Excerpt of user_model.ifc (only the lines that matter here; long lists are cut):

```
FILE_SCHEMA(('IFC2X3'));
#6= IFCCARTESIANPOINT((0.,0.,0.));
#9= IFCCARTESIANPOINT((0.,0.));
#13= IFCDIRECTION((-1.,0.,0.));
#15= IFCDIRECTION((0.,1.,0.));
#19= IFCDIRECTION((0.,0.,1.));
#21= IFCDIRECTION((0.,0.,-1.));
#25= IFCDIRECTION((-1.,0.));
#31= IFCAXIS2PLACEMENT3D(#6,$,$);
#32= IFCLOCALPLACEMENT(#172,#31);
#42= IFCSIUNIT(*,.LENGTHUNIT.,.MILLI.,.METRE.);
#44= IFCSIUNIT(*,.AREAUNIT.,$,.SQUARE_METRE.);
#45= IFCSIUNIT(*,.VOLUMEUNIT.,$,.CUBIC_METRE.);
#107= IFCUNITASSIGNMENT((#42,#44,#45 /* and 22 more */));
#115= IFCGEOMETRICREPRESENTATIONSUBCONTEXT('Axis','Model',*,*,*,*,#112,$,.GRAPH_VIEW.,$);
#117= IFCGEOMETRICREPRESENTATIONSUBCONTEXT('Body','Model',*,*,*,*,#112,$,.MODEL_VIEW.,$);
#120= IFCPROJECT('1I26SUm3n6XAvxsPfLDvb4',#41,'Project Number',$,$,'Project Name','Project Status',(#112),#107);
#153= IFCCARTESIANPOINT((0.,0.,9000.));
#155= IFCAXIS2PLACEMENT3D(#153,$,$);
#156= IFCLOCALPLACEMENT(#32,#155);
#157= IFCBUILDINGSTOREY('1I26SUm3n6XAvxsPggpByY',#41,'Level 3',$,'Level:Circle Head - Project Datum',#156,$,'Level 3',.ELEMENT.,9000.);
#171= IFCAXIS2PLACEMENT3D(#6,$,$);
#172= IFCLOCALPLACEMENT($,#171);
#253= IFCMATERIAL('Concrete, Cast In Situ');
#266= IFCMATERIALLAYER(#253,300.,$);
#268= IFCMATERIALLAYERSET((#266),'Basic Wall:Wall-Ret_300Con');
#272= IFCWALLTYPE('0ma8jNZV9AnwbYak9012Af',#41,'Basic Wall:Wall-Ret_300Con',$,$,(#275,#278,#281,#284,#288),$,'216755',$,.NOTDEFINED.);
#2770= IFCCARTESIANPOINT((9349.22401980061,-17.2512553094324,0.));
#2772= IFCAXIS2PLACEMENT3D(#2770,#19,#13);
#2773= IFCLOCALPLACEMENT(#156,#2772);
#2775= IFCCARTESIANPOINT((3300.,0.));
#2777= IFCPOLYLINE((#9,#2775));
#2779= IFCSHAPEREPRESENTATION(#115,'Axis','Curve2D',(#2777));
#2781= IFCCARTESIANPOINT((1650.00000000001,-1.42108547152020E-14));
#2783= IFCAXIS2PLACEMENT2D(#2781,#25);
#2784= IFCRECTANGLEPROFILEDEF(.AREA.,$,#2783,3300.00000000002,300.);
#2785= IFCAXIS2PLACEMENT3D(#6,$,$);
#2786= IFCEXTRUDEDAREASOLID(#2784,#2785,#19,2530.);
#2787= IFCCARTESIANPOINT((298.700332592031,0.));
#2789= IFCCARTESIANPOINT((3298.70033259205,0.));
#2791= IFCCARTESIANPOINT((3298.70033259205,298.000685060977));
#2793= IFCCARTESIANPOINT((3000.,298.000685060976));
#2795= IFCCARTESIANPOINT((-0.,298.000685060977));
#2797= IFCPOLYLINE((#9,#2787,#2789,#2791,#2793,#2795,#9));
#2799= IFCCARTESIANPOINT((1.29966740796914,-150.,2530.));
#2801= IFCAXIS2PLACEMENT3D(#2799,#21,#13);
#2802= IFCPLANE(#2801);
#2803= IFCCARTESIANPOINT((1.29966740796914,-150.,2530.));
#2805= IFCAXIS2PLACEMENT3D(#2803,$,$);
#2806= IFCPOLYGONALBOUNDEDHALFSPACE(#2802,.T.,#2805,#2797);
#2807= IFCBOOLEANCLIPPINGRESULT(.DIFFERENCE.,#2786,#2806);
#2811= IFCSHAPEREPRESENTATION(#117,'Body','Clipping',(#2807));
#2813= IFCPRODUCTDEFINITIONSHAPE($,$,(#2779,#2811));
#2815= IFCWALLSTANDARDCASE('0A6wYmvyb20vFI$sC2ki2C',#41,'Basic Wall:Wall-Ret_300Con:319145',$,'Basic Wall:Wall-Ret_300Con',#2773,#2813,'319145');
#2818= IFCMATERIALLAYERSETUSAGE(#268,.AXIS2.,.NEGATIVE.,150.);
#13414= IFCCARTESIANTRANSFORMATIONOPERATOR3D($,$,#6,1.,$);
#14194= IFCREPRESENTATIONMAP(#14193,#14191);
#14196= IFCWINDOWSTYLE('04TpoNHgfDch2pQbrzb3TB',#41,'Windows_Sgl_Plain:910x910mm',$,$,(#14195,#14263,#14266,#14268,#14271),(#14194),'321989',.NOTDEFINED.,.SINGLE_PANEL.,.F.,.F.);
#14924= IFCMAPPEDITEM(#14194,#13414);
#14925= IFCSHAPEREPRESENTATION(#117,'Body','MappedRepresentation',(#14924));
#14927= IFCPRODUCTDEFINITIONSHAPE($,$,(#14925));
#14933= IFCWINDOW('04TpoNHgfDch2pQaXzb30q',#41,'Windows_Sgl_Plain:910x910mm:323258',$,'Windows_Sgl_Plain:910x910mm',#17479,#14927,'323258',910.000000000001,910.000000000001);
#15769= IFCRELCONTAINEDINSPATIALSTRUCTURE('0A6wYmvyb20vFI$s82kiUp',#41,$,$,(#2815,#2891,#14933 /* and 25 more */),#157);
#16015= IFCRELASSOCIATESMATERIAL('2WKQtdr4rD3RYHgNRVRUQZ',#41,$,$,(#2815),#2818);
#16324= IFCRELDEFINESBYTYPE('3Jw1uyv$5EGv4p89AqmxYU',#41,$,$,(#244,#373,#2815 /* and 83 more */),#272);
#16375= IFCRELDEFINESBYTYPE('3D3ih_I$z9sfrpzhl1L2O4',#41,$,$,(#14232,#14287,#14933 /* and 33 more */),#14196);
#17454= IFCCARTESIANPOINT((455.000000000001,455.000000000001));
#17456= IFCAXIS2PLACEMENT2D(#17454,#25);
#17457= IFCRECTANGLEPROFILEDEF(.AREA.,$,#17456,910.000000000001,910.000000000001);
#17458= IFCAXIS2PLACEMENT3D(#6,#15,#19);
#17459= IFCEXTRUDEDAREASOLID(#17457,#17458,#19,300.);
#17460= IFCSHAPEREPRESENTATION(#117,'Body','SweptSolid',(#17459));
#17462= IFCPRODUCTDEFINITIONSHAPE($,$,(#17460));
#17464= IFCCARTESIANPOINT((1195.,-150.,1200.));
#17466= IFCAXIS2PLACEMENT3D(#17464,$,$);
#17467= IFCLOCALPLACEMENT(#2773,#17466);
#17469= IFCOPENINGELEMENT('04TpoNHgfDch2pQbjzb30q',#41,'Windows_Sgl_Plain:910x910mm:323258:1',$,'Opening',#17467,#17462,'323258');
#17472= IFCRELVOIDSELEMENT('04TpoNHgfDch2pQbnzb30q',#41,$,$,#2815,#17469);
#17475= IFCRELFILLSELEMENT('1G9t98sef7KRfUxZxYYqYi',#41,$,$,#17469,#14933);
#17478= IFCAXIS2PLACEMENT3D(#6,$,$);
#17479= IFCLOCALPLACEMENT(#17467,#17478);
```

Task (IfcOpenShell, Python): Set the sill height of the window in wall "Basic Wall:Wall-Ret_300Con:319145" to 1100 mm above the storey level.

```python
import numpy as np
import ifcopenshell
import ifcopenshell.api.geometry
import ifcopenshell.geom
import ifcopenshell.util.element
import ifcopenshell.util.placement
import ifcopenshell.util.shape
import ifcopenshell.util.unit

model = ifcopenshell.open("user_model.ifc")
unit_scale = ifcopenshell.util.unit.calculate_unit_scale(model)

window = model.by_guid("04TpoNHgfDch2pQaXzb30q")
opening = window.FillsVoids[0].RelatingOpeningElement
storey = ifcopenshell.util.element.get_container(window, ifc_class="IfcBuildingStorey")
level = ifcopenshell.util.placement.get_local_placement(storey.ObjectPlacement)[2, 3]

# The opening's origin need not be at the sill, so measure its lowest point.
shape = ifcopenshell.geom.create_shape(ifcopenshell.geom.settings(), opening)
bottom = ifcopenshell.util.shape.get_shape_bottom_elevation(shape, shape.geometry) / unit_scale
dz = level + 1.1 / unit_scale - bottom

shift = np.array([0.0, 0.0, dz])
# The window is placed relative to its opening, so it follows when the opening moves.
matrix = ifcopenshell.util.placement.get_local_placement(opening.ObjectPlacement)
matrix[:3, 3] += shift
ifcopenshell.api.geometry.edit_object_placement(
    model, product=opening, matrix=matrix, is_si=False, should_transform_children=True
)

print(f"moved by {dz * unit_scale:+.3f} m")

model.write("user_model_edited.ifc")
```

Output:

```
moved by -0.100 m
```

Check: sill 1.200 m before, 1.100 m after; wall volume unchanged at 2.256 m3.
